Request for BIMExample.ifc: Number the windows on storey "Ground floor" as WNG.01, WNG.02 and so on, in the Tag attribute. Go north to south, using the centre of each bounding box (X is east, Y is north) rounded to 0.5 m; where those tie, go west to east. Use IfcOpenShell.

First a look at what the model holds.

```python
import ifcopenshell
import ifcopenshell.util.element
import ifcopenshell.util.placement

model = ifcopenshell.open("BIMExample.ifc")
print(model.schema)
storey = next(s for s in model.by_type("IfcBuildingStorey") if s.Name == "Ground floor")
windows = [e for e in ifcopenshell.util.element.get_decomposition(storey) if e.is_a("IfcWindow")]
for e in sorted(windows, key=lambda e: e.id()):
    origin = ifcopenshell.util.placement.get_local_placement(e.ObjectPlacement)[:3, 3]
    print(e.id(), e.Tag, e.Name, origin.round(2) + 0.0, sep=" | ")
```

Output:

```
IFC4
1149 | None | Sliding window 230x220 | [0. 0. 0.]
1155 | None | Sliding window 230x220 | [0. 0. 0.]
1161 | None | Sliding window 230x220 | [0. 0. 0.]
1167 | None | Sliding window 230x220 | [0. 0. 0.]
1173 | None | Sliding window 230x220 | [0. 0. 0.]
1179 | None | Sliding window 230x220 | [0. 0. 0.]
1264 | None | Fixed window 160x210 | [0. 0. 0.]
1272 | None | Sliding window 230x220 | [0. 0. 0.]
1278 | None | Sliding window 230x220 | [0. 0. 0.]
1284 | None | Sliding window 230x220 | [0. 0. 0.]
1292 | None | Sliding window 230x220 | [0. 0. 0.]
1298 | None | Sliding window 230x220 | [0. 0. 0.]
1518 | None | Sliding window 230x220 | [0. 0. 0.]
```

```python
import ifcopenshell
import ifcopenshell.geom
import ifcopenshell.util.element
import ifcopenshell.util.shape

model = ifcopenshell.open("BIMExample.ifc")
settings = ifcopenshell.geom.settings()
settings.set("use-world-coords", True)


def centre(element):
    shape = ifcopenshell.geom.create_shape(settings, element)
    return ifcopenshell.util.shape.get_bbox_centroid(shape.geometry)


storey = next(s for s in model.by_type("IfcBuildingStorey") if s.Name == "Ground floor")
windows = [e for e in ifcopenshell.util.element.get_decomposition(storey) if e.is_a("IfcWindow")]

# Insertion points can sit at a corner or the storey origin, so sort by the geometry (in metres).
centres = {e: centre(e) for e in windows}
windows.sort(key=lambda e: (-round(centres[e][1] / 0.5), centres[e][0]))

for i, e in enumerate(windows, start=1):
    number = f"WNG.{i:02d}"
    e.Tag = number
    print(e.id(), number)

model.write("BIMExample_edited.ifc")
```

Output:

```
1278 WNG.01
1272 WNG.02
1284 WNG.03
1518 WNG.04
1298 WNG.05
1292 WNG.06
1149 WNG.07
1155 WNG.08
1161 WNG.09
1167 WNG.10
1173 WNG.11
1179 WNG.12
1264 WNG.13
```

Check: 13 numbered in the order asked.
